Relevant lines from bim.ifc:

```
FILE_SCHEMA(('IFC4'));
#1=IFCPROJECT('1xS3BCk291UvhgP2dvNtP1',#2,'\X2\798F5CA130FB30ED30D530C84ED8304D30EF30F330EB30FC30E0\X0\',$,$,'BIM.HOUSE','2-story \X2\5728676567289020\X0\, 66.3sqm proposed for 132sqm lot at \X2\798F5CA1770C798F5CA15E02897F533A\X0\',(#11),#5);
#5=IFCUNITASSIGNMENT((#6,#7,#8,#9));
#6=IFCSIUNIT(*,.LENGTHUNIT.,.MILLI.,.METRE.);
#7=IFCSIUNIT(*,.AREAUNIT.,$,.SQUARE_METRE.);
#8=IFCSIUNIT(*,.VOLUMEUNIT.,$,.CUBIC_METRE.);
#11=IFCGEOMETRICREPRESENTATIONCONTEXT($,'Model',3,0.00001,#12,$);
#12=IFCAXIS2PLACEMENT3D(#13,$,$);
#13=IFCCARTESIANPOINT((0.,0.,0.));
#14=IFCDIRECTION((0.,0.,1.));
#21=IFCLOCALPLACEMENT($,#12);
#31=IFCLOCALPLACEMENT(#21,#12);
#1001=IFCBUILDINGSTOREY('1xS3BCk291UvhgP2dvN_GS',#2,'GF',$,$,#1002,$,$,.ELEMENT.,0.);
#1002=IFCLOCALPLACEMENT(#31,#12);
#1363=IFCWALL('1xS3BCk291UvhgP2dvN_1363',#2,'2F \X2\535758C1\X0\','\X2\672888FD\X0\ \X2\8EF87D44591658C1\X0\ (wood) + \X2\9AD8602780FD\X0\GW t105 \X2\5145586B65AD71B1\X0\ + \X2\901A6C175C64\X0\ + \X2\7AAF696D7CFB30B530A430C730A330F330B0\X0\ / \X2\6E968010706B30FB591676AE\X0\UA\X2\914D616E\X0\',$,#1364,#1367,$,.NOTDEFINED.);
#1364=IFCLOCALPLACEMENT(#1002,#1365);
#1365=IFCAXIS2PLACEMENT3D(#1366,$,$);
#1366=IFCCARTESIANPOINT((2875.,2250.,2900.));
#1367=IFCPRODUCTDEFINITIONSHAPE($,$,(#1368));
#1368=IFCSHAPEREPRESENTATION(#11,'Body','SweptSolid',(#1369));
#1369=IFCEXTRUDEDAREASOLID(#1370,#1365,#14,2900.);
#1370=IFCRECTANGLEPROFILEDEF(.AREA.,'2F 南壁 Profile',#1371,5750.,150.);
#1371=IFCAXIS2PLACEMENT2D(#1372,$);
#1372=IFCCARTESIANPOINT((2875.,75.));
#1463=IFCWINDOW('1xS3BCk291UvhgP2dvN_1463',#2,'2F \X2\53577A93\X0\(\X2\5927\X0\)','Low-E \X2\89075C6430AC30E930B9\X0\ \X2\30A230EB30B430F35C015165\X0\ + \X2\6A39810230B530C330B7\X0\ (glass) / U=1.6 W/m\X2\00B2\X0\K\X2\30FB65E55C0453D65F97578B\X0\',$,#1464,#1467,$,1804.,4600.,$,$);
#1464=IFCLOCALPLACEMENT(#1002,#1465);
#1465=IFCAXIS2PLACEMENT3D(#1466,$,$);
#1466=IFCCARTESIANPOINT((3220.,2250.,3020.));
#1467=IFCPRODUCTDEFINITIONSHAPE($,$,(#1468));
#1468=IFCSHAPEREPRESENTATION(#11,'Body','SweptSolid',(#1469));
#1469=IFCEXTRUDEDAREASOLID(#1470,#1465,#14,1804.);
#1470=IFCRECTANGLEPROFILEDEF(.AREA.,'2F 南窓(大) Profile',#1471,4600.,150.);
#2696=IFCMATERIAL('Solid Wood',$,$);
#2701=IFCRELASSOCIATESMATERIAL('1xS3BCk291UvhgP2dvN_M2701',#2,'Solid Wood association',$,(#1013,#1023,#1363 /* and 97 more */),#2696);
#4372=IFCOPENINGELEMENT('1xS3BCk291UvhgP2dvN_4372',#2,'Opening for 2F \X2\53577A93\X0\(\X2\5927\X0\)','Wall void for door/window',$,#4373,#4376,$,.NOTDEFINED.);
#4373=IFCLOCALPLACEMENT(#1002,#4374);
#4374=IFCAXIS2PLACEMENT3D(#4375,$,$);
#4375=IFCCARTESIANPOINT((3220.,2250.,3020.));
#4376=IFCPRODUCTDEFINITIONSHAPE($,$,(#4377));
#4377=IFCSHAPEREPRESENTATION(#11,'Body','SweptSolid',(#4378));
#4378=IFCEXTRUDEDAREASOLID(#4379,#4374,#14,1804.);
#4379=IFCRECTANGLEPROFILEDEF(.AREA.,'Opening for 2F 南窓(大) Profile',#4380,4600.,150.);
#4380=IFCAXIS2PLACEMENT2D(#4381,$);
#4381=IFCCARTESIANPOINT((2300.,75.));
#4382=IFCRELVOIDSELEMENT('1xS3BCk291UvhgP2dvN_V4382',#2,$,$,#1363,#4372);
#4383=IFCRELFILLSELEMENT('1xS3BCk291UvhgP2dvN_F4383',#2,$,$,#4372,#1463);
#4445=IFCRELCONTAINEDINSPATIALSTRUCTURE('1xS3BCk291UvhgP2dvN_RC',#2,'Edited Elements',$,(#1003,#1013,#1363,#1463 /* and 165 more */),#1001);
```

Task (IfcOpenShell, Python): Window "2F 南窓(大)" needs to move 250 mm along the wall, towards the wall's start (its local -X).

```python
import ifcopenshell
import ifcopenshell.api.geometry
import ifcopenshell.util.placement

model = ifcopenshell.open("bim.ifc")

window = model.by_guid("1xS3BCk291UvhgP2dvN_1463")
opening = window.FillsVoids[0].RelatingOpeningElement
wall = opening.VoidsElements[0].RelatingBuildingElement

wall_matrix = ifcopenshell.util.placement.get_local_placement(wall.ObjectPlacement)
shift = wall_matrix[:3, 0] * -250.0
before = ifcopenshell.util.placement.get_local_placement(window.ObjectPlacement)[:3, 3].copy()

# The window is not placed relative to its opening, so move both.
for product in (opening, window):
    matrix = ifcopenshell.util.placement.get_local_placement(product.ObjectPlacement)
    matrix[:3, 3] += shift
    ifcopenshell.api.geometry.edit_object_placement(model, product=product, matrix=matrix, is_si=False)

after = ifcopenshell.util.placement.get_local_placement(window.ObjectPlacement)[:3, 3]
print("window moved by", (after - before).round(3) + 0.0)

model.write("bim_v2.ifc")
```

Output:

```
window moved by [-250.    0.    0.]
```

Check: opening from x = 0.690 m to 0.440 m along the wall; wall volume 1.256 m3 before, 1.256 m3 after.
